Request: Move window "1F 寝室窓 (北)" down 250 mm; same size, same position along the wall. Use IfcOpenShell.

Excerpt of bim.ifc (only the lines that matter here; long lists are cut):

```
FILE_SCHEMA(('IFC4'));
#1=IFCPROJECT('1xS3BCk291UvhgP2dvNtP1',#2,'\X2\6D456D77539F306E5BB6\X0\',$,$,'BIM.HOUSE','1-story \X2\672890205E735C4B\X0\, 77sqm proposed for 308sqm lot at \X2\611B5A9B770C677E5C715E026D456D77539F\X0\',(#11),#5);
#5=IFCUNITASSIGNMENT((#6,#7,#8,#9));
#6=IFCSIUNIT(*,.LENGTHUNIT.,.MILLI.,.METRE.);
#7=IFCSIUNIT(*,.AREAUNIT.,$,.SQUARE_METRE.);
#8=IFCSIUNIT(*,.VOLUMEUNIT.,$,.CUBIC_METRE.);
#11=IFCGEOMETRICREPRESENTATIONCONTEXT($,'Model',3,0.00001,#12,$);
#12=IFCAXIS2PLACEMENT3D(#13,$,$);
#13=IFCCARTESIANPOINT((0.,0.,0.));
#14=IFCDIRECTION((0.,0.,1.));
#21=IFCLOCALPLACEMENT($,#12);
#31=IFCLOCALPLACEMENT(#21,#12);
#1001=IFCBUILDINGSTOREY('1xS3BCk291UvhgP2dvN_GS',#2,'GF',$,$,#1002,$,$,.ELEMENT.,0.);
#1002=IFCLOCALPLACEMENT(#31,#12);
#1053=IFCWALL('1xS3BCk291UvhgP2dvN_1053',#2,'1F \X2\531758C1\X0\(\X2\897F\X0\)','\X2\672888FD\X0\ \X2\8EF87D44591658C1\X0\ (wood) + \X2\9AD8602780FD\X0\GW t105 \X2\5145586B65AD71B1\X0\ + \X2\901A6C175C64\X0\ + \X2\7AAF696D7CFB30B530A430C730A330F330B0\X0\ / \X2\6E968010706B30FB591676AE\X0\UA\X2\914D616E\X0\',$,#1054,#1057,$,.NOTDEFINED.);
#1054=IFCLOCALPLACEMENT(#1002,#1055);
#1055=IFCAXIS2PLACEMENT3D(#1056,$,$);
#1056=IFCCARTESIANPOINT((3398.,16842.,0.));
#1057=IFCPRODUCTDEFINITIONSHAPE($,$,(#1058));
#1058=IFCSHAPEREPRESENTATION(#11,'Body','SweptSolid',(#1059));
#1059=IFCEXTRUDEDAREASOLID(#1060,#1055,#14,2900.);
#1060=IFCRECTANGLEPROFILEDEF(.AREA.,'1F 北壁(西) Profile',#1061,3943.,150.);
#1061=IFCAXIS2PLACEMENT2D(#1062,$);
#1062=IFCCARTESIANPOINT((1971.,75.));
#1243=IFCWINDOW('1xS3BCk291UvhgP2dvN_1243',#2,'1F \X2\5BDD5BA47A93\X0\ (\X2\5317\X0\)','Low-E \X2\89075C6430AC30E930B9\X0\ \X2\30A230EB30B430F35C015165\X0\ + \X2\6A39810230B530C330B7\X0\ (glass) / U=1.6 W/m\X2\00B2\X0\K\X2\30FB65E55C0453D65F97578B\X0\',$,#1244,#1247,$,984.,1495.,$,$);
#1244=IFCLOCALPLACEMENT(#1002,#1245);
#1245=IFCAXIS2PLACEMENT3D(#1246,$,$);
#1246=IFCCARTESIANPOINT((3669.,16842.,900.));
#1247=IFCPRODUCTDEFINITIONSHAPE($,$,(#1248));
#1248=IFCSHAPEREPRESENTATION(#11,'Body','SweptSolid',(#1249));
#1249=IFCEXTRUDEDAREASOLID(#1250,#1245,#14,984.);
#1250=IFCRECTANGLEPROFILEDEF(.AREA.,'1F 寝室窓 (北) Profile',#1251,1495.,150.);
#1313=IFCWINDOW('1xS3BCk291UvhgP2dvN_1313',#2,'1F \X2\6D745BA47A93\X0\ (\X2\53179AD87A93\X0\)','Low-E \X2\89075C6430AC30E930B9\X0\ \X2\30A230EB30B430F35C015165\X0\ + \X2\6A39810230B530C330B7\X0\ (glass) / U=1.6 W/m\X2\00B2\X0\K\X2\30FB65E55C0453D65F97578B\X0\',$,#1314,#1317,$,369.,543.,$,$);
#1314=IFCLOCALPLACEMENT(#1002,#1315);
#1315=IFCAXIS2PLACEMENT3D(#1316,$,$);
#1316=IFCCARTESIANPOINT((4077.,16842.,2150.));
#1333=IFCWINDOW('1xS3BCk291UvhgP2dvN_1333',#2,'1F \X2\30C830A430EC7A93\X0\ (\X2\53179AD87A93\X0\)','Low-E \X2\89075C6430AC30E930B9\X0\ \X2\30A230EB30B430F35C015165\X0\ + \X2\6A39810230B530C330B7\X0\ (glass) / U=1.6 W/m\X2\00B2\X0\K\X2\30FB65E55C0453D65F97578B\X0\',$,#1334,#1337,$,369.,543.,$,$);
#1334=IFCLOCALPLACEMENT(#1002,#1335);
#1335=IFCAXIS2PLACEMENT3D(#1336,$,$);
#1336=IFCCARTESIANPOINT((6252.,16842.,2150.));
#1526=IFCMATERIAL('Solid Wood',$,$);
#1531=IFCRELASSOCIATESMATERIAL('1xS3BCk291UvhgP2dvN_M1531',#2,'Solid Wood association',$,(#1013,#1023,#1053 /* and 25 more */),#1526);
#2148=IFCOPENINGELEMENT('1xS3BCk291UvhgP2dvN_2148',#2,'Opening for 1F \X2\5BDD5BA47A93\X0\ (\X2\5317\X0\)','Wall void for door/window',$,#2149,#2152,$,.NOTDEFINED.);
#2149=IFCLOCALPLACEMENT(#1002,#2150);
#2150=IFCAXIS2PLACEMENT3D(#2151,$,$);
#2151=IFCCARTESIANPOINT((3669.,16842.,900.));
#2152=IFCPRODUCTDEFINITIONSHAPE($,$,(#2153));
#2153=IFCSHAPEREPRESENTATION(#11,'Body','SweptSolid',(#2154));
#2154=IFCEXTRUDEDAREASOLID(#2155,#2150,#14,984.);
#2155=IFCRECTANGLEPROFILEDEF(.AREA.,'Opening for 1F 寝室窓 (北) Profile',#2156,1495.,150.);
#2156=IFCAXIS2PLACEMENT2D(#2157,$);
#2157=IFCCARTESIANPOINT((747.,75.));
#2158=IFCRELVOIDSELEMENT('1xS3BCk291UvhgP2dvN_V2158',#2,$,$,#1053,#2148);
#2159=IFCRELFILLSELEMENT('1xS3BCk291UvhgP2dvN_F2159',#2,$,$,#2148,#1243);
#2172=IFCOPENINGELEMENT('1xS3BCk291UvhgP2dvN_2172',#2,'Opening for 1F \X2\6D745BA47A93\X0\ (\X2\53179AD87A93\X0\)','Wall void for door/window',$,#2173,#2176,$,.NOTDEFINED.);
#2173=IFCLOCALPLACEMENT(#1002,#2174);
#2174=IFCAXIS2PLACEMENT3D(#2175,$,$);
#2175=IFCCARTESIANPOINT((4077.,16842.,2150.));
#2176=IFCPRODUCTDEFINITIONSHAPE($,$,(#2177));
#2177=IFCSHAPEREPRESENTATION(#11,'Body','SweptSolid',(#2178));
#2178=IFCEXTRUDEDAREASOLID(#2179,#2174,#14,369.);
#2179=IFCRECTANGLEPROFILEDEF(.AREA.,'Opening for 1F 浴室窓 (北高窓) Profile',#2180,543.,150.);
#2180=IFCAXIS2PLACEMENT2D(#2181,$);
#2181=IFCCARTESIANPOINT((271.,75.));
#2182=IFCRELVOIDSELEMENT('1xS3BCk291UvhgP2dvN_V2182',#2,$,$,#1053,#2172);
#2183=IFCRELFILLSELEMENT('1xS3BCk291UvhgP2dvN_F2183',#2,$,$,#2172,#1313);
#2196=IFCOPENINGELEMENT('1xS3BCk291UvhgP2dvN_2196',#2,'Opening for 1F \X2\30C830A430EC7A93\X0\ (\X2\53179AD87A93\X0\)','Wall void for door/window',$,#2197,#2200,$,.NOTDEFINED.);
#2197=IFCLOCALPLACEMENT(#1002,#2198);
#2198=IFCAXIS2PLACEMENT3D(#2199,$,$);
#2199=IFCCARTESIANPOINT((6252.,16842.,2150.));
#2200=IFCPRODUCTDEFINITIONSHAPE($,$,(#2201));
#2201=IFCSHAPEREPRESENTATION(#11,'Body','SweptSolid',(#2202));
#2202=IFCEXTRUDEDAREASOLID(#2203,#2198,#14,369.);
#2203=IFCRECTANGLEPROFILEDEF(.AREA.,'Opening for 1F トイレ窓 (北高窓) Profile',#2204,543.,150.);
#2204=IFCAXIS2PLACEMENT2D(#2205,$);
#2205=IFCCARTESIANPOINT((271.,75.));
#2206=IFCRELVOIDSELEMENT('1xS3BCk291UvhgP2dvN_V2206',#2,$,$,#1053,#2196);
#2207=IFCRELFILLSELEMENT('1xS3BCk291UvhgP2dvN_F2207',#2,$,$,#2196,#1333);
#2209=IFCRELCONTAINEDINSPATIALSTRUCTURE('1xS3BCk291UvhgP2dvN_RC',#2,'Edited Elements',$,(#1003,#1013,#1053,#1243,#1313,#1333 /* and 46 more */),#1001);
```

```python
import numpy as np
import ifcopenshell
import ifcopenshell.api.geometry
import ifcopenshell.util.placement
import ifcopenshell.util.unit

model = ifcopenshell.open("bim.ifc")
unit_scale = ifcopenshell.util.unit.calculate_unit_scale(model)

window = model.by_id(1243)
opening = window.FillsVoids[0].RelatingOpeningElement
dz = -0.25 / unit_scale

shift = np.array([0.0, 0.0, dz])
# The window is not placed relative to its opening, so move both.
for product in (opening, window):
    matrix = ifcopenshell.util.placement.get_local_placement(product.ObjectPlacement)
    matrix[:3, 3] += shift
    ifcopenshell.api.geometry.edit_object_placement(model, product=product, matrix=matrix, is_si=False)

print(f"moved by {dz * unit_scale:+.3f} m")

model.write("bim-out.ifc")
```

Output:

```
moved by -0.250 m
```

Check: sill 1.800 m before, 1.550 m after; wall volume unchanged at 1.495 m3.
